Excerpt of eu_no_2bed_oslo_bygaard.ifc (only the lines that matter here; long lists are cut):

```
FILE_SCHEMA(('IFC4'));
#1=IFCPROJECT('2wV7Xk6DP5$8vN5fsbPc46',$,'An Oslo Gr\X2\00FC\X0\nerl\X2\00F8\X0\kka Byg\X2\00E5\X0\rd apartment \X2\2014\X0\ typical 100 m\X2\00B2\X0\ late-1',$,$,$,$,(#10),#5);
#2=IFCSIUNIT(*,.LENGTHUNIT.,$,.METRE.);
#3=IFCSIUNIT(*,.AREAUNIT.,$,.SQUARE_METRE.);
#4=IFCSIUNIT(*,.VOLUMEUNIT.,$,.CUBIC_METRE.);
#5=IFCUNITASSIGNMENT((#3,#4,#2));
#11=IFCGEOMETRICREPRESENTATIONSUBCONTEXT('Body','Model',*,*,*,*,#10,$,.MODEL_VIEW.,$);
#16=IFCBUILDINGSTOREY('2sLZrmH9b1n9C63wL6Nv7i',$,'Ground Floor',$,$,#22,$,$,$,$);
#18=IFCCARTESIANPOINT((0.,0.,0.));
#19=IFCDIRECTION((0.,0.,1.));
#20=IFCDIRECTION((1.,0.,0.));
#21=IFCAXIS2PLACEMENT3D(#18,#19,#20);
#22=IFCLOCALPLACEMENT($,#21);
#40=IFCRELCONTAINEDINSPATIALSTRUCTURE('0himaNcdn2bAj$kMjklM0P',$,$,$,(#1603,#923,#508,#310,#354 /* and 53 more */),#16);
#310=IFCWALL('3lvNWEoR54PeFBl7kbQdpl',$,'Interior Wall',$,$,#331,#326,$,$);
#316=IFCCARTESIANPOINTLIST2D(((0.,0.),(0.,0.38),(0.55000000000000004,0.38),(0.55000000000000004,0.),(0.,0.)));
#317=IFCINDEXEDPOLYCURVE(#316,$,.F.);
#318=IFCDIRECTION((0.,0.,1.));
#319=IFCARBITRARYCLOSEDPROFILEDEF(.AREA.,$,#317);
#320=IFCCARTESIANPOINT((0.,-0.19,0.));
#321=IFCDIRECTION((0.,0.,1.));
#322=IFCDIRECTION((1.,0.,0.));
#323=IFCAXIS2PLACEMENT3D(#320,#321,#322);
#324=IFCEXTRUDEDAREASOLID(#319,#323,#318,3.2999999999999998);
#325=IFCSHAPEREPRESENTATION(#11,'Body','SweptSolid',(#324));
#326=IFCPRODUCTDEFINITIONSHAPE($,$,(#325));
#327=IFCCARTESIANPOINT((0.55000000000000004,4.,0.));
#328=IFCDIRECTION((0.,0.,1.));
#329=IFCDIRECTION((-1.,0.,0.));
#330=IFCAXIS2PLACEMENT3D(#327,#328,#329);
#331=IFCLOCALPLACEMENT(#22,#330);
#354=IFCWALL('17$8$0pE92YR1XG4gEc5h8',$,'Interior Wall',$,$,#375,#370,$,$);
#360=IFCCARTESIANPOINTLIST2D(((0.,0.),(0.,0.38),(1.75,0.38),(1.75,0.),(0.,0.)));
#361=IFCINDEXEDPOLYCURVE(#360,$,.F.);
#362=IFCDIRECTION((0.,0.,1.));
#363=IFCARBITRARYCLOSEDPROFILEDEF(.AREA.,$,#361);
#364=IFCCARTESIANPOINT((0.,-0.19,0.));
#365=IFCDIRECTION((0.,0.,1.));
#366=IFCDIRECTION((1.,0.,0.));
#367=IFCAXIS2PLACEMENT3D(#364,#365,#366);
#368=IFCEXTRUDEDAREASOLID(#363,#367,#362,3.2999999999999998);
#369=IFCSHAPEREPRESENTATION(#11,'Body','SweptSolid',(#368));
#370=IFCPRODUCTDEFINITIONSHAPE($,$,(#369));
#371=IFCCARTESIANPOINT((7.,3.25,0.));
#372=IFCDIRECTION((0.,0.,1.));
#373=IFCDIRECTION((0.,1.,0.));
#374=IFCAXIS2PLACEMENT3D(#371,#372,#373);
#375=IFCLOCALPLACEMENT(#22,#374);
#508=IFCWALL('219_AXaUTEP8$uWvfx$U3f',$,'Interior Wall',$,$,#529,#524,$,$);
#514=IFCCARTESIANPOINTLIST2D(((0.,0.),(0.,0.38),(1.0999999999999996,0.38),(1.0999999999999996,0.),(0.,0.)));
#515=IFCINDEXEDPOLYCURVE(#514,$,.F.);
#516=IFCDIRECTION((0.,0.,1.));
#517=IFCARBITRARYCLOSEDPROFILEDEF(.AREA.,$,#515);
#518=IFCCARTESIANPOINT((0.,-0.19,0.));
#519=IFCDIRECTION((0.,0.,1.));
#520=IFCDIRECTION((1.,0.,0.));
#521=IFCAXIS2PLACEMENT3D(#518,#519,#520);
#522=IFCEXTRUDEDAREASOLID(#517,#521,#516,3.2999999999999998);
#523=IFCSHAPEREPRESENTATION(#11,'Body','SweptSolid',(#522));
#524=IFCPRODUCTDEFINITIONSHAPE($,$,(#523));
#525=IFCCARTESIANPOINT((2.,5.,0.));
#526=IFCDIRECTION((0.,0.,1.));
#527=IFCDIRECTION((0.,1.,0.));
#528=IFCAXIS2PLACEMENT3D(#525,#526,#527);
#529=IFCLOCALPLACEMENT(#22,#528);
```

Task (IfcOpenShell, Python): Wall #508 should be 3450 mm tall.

```python
import ifcopenshell
import ifcopenshell.geom
import ifcopenshell.util.representation
import ifcopenshell.util.shape

model = ifcopenshell.open("eu_no_2bed_oslo_bygaard.ifc")
settings = ifcopenshell.geom.settings()


def volume(element):
    """Net volume in cubic metres, openings subtracted."""
    shape = ifcopenshell.geom.create_shape(settings, element)
    return ifcopenshell.util.shape.get_volume(shape.geometry)


wall = model.by_guid("219_AXaUTEP8$uWvfx$U3f")
before = volume(wall)

body = ifcopenshell.util.representation.get_representation(wall, "Model", "Body")
solid = body.Items[0]
old_height = solid.Depth
solid.Depth = 3.45
after = volume(wall)

print(f"height {old_height:g} -> {solid.Depth:g}, volume {before:.3f} -> {after:.3f} m3")

model.write("eu_no_2bed_oslo_bygaard_v2.ifc")
```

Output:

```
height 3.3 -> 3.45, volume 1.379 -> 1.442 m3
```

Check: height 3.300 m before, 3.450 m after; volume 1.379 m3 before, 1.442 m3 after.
